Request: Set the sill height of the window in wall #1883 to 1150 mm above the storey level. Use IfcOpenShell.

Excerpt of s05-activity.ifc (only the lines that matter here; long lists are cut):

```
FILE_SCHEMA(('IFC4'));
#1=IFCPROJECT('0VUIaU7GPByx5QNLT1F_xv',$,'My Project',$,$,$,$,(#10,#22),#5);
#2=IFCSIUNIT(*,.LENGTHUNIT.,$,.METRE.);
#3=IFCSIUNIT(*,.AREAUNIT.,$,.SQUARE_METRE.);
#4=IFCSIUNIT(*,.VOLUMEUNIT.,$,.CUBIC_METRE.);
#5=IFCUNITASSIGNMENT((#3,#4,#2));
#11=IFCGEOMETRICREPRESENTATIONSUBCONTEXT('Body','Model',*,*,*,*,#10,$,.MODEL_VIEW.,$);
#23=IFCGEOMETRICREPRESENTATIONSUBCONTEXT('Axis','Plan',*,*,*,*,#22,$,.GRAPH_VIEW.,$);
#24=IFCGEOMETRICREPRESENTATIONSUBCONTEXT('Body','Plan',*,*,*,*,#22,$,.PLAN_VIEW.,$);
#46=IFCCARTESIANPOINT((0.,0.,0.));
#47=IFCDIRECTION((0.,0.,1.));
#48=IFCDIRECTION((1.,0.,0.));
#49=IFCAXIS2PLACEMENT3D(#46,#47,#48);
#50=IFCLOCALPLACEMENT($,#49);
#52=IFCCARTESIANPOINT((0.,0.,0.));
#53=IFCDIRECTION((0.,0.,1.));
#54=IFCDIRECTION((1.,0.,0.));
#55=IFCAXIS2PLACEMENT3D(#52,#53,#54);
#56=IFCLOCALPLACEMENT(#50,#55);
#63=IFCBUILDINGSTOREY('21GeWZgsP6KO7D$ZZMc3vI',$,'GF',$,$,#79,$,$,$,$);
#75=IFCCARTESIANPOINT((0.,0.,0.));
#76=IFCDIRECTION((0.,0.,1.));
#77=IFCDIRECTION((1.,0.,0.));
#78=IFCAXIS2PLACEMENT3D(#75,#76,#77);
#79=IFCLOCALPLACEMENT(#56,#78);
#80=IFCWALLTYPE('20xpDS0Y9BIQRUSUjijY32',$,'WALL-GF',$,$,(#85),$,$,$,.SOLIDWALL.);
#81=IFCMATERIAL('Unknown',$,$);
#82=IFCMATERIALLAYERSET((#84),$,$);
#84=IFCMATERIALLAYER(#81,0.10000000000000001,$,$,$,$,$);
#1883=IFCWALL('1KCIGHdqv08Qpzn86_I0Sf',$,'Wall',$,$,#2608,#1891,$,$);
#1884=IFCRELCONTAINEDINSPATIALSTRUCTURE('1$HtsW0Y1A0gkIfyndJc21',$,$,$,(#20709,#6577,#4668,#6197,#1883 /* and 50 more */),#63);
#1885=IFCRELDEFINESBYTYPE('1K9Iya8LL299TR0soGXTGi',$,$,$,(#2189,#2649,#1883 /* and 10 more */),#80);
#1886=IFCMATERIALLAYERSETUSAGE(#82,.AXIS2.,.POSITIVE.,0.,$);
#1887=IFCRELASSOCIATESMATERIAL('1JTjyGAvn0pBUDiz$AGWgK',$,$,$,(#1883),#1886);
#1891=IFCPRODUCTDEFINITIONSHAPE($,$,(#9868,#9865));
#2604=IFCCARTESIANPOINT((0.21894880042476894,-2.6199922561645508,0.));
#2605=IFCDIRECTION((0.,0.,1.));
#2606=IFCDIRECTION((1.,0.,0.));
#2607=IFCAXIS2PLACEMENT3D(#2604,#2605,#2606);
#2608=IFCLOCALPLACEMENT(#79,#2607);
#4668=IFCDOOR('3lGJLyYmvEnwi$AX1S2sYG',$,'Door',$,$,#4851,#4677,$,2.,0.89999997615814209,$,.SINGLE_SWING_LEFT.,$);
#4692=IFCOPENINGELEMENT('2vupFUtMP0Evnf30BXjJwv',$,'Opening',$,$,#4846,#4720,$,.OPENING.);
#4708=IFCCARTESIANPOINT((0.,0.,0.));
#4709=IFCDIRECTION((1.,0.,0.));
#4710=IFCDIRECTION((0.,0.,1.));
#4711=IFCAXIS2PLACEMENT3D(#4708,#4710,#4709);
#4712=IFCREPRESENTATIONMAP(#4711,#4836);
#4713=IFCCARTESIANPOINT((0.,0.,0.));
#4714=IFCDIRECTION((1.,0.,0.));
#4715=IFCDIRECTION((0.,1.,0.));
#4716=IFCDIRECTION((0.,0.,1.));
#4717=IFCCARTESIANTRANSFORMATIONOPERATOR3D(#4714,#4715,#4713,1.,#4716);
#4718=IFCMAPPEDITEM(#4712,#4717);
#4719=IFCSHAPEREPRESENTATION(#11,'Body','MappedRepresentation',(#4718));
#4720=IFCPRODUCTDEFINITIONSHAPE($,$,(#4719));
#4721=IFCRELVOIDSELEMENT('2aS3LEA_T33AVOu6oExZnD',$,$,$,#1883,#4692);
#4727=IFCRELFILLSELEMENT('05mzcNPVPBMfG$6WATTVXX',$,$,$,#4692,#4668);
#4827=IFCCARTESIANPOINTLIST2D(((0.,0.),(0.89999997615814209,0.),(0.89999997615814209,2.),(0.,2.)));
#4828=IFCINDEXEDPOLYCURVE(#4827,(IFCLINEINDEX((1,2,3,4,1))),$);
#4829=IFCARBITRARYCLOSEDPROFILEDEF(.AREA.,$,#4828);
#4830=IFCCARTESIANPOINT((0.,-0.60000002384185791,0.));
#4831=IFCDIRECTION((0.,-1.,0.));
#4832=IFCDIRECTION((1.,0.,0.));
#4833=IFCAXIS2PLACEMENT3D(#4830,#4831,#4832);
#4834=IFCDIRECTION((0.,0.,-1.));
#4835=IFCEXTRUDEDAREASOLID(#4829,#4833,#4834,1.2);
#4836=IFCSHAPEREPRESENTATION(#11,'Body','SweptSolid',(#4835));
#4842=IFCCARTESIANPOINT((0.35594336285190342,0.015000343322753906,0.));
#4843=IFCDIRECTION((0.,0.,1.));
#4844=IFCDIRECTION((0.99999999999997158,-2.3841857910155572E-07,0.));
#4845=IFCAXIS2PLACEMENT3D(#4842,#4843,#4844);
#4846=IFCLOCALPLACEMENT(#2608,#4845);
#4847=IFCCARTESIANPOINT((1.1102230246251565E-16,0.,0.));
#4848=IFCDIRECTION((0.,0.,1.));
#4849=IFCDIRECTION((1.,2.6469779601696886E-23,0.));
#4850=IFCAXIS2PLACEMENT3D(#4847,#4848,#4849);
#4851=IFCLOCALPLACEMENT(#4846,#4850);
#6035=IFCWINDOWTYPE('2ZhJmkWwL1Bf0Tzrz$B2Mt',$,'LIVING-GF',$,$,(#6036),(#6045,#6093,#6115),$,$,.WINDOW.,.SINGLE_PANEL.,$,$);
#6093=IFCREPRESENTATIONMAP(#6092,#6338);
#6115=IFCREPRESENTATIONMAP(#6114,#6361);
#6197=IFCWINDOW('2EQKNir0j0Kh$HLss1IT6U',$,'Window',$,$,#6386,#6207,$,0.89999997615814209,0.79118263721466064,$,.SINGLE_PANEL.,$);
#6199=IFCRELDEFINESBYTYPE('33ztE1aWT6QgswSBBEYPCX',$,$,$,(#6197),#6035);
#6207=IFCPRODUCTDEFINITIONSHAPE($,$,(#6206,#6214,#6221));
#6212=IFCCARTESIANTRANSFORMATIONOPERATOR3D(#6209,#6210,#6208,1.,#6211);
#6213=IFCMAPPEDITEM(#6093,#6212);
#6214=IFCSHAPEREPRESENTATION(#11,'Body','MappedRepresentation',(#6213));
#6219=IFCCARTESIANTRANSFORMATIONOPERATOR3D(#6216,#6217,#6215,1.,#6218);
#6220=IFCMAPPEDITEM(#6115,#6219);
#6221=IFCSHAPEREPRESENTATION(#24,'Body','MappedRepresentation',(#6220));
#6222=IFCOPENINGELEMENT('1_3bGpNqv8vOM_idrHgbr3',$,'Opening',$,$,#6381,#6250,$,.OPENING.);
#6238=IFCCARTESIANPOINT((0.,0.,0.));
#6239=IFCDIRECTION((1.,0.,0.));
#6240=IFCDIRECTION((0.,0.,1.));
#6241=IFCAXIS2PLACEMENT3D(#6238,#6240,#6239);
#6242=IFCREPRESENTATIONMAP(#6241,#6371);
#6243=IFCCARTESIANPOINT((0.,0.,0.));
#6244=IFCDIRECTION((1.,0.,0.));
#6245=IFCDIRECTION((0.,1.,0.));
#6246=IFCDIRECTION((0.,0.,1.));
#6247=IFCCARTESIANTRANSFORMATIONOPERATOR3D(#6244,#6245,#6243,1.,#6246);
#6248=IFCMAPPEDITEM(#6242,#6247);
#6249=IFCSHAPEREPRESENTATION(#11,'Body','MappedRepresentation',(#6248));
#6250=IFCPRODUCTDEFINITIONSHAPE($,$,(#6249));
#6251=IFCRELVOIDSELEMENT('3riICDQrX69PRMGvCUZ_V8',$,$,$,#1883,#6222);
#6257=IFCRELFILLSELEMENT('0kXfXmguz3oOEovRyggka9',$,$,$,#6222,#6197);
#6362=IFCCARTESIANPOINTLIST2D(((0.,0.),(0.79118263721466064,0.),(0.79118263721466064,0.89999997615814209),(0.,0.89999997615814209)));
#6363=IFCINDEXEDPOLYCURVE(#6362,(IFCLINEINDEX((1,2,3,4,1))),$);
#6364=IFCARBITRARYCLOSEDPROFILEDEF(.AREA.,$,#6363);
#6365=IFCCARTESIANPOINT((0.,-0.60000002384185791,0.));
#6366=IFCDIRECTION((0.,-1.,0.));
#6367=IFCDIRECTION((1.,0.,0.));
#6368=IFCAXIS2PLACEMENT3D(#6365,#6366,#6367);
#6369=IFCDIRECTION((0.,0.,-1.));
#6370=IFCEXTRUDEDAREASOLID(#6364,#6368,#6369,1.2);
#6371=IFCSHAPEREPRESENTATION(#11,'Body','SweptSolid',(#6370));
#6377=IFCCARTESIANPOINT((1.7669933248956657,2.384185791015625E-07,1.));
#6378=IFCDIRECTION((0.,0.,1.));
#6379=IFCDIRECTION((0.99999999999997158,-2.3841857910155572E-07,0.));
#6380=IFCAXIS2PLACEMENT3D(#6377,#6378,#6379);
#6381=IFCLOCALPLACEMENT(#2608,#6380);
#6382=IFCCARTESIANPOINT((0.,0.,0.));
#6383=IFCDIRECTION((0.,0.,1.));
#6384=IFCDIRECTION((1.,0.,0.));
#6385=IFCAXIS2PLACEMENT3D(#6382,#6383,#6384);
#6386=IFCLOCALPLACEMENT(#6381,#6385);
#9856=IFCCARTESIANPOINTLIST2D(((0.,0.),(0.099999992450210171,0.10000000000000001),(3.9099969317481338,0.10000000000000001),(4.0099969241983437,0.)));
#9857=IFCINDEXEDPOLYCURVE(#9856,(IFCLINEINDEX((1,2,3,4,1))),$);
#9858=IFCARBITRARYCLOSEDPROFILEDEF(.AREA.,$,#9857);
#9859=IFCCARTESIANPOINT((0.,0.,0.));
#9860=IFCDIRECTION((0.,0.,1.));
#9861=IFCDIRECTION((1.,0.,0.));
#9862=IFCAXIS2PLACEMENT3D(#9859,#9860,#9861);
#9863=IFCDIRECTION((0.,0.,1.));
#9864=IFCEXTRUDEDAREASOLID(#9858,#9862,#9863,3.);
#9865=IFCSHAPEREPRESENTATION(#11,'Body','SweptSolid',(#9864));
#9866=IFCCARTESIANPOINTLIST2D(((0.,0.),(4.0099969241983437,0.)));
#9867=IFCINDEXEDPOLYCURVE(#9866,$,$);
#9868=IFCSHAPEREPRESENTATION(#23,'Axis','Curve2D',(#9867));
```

```python
import numpy as np
import ifcopenshell
import ifcopenshell.api.geometry
import ifcopenshell.geom
import ifcopenshell.util.element
import ifcopenshell.util.placement
import ifcopenshell.util.shape
import ifcopenshell.util.unit

model = ifcopenshell.open("s05-activity.ifc")
unit_scale = ifcopenshell.util.unit.calculate_unit_scale(model)

window = model.by_guid("2EQKNir0j0Kh$HLss1IT6U")
opening = window.FillsVoids[0].RelatingOpeningElement
storey = ifcopenshell.util.element.get_container(window, ifc_class="IfcBuildingStorey")
level = ifcopenshell.util.placement.get_local_placement(storey.ObjectPlacement)[2, 3]

# The opening's origin need not be at the sill, so measure its lowest point.
shape = ifcopenshell.geom.create_shape(ifcopenshell.geom.settings(), opening)
bottom = ifcopenshell.util.shape.get_shape_bottom_elevation(shape, shape.geometry) / unit_scale
dz = level + 1.15 / unit_scale - bottom

shift = np.array([0.0, 0.0, dz])
# The window is placed relative to its opening, so it follows when the opening moves.
matrix = ifcopenshell.util.placement.get_local_placement(opening.ObjectPlacement)
matrix[:3, 3] += shift
ifcopenshell.api.geometry.edit_object_placement(
    model, product=opening, matrix=matrix, is_si=False, should_transform_children=True
)

print(f"moved by {dz * unit_scale:+.3f} m")

model.write("s05-activity_edited.ifc")
```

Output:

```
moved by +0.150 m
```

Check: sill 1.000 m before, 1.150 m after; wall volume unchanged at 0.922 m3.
